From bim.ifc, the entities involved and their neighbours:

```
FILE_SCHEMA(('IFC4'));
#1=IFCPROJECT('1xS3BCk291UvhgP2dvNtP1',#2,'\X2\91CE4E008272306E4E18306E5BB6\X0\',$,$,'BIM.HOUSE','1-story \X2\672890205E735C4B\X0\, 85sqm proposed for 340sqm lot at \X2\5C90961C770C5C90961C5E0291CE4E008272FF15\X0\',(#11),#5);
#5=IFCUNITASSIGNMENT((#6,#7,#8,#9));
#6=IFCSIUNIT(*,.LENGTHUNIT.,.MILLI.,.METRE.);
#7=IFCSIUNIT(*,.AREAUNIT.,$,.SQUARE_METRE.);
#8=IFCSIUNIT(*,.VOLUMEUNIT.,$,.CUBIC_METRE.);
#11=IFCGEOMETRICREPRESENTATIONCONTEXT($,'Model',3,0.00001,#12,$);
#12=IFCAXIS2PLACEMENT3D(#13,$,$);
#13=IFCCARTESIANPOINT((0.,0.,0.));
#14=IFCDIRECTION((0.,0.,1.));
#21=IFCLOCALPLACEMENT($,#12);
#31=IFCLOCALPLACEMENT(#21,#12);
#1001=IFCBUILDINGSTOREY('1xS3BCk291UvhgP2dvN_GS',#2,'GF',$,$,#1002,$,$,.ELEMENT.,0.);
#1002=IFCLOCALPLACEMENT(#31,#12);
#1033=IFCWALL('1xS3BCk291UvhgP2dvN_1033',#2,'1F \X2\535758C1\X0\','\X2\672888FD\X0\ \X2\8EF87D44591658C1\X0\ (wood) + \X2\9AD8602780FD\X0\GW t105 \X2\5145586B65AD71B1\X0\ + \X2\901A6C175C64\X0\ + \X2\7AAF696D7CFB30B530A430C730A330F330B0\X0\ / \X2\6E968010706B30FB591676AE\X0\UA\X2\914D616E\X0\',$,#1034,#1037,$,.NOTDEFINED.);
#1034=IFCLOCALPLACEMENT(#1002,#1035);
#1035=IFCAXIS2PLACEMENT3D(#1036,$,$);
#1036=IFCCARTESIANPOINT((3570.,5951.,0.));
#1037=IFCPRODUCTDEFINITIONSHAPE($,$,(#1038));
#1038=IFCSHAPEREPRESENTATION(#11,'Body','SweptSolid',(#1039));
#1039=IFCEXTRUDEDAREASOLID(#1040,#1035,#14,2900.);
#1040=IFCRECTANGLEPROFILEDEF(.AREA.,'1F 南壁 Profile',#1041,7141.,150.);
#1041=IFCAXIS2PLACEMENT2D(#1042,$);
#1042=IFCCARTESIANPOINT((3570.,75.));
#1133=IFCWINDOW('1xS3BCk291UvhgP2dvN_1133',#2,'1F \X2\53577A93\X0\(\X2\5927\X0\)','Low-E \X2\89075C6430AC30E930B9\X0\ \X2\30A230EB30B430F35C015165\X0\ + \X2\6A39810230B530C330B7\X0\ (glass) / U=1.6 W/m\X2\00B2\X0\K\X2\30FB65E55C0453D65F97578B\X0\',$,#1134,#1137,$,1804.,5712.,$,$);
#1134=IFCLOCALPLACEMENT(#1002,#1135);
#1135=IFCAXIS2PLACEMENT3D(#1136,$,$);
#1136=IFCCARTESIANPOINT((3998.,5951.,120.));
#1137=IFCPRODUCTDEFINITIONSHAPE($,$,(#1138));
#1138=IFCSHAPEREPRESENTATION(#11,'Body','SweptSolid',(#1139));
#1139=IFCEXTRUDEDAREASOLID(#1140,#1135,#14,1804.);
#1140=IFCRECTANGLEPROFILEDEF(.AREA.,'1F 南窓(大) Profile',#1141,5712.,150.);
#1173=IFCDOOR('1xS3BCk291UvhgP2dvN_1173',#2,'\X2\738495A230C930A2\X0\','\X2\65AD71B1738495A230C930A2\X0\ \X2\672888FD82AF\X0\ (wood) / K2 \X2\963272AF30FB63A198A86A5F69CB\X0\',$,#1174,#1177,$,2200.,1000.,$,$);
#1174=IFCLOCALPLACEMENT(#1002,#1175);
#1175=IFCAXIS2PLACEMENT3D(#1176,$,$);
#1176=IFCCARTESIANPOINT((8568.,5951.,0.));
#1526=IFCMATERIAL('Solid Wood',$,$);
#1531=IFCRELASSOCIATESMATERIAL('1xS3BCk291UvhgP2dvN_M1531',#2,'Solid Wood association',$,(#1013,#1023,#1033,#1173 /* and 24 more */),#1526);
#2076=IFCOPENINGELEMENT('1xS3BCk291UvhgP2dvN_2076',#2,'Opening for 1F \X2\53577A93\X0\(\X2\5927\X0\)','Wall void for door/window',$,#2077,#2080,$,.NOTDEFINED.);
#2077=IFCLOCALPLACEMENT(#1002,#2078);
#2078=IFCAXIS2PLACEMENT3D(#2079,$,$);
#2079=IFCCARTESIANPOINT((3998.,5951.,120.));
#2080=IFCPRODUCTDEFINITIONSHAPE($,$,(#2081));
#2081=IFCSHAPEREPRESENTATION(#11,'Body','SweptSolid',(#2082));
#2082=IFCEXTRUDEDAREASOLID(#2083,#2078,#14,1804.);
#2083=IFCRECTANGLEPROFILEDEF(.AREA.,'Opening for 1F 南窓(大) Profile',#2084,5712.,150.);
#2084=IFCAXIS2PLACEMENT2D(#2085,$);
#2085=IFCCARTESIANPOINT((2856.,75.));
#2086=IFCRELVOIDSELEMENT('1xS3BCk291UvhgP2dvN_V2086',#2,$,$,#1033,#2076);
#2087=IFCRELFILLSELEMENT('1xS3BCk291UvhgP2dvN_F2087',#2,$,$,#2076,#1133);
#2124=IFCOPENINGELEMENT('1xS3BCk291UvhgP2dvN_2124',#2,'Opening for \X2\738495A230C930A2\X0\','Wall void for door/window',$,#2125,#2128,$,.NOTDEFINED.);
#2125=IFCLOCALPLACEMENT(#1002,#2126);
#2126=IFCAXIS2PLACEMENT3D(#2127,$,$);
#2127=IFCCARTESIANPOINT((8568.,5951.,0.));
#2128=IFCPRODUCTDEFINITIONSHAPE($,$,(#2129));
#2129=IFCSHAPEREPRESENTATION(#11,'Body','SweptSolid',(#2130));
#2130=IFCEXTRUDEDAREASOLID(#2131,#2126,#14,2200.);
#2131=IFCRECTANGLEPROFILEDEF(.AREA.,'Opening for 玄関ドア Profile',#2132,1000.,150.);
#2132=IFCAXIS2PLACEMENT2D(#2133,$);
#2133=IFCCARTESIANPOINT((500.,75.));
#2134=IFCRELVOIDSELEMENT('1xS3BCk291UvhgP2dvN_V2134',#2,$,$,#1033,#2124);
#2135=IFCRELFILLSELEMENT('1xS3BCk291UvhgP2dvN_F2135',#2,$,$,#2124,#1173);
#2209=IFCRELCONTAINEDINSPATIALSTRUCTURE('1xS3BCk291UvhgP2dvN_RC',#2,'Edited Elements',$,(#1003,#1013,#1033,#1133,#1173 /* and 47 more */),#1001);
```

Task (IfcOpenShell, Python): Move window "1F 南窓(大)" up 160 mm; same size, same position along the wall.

```python
import numpy as np
import ifcopenshell
import ifcopenshell.api.geometry
import ifcopenshell.util.placement
import ifcopenshell.util.unit

model = ifcopenshell.open("bim.ifc")
unit_scale = ifcopenshell.util.unit.calculate_unit_scale(model)

window = model.by_id(1133)
opening = window.FillsVoids[0].RelatingOpeningElement
dz = 160.0

shift = np.array([0.0, 0.0, dz])
# The window is not placed relative to its opening, so move both.
for product in (opening, window):
    matrix = ifcopenshell.util.placement.get_local_placement(product.ObjectPlacement)
    matrix[:3, 3] += shift
    ifcopenshell.api.geometry.edit_object_placement(model, product=product, matrix=matrix, is_si=False)

print(f"moved by {dz * unit_scale:+.3f} m")

model.write("bim_rev.ifc")
```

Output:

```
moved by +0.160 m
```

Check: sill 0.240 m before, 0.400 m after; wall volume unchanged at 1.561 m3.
